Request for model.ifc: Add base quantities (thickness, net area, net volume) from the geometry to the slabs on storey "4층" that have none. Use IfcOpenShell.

First a look at what the model holds.

```python
import ifcopenshell
import ifcopenshell.util.element
import ifcopenshell.util.unit

model = ifcopenshell.open("model.ifc")
print(model.schema)
for unit_type in ("LENGTHUNIT", "AREAUNIT", "VOLUMEUNIT"):
    print(unit_type, ifcopenshell.util.unit.calculate_unit_scale(model, unit_type))
storey = next(s for s in model.by_type("IfcBuildingStorey") if s.Name == "4층")
slabs = [e for e in ifcopenshell.util.element.get_decomposition(storey) if e.is_a("IfcSlab")]
for e in sorted(slabs, key=lambda e: e.id()):
    print(e.id(), e.is_a(), e.Name, list(ifcopenshell.util.element.get_psets(e, qtos_only=True)), sep=" | ")
```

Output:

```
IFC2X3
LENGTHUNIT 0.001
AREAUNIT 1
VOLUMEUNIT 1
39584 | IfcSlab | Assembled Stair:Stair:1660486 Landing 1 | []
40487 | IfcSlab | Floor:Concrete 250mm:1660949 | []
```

```python
import ifcopenshell
import ifcopenshell.api.pset
import ifcopenshell.geom
import ifcopenshell.util.element
import ifcopenshell.util.shape
import ifcopenshell.util.unit

model = ifcopenshell.open("model.ifc")
unit_scale = ifcopenshell.util.unit.calculate_unit_scale(model)
area_scale = ifcopenshell.util.unit.calculate_unit_scale(model, "AREAUNIT")
volume_scale = ifcopenshell.util.unit.calculate_unit_scale(model, "VOLUMEUNIT")
settings = ifcopenshell.geom.settings()

storey = next(s for s in model.by_type("IfcBuildingStorey") if s.Name == "4층")
slabs = [e for e in ifcopenshell.util.element.get_decomposition(storey) if e.is_a("IfcSlab")]

for e in sorted(slabs, key=lambda e: e.id()):
    if ifcopenshell.util.element.get_psets(e, qtos_only=True, should_inherit=False):
        continue
    # Geometry comes back in metres, in the element's own axes.
    shape = ifcopenshell.geom.create_shape(settings, e)
    values = {
        "Width": ifcopenshell.util.shape.get_z(shape.geometry) / unit_scale,
        "NetArea": ifcopenshell.util.shape.get_footprint_area(shape.geometry) / area_scale,
        "NetVolume": ifcopenshell.util.shape.get_volume(shape.geometry) / volume_scale,
    }
    qto = ifcopenshell.api.pset.add_qto(model, product=e, name="BaseQuantities")
    ifcopenshell.api.pset.edit_qto(model, qto=qto, properties=values)
    print(e.id(), {k: round(v, 3) for k, v in values.items()})

model.write("model_edited.ifc")
```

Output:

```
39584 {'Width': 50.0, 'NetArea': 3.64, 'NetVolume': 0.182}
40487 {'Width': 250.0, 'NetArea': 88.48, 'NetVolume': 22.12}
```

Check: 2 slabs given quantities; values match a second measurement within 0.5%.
